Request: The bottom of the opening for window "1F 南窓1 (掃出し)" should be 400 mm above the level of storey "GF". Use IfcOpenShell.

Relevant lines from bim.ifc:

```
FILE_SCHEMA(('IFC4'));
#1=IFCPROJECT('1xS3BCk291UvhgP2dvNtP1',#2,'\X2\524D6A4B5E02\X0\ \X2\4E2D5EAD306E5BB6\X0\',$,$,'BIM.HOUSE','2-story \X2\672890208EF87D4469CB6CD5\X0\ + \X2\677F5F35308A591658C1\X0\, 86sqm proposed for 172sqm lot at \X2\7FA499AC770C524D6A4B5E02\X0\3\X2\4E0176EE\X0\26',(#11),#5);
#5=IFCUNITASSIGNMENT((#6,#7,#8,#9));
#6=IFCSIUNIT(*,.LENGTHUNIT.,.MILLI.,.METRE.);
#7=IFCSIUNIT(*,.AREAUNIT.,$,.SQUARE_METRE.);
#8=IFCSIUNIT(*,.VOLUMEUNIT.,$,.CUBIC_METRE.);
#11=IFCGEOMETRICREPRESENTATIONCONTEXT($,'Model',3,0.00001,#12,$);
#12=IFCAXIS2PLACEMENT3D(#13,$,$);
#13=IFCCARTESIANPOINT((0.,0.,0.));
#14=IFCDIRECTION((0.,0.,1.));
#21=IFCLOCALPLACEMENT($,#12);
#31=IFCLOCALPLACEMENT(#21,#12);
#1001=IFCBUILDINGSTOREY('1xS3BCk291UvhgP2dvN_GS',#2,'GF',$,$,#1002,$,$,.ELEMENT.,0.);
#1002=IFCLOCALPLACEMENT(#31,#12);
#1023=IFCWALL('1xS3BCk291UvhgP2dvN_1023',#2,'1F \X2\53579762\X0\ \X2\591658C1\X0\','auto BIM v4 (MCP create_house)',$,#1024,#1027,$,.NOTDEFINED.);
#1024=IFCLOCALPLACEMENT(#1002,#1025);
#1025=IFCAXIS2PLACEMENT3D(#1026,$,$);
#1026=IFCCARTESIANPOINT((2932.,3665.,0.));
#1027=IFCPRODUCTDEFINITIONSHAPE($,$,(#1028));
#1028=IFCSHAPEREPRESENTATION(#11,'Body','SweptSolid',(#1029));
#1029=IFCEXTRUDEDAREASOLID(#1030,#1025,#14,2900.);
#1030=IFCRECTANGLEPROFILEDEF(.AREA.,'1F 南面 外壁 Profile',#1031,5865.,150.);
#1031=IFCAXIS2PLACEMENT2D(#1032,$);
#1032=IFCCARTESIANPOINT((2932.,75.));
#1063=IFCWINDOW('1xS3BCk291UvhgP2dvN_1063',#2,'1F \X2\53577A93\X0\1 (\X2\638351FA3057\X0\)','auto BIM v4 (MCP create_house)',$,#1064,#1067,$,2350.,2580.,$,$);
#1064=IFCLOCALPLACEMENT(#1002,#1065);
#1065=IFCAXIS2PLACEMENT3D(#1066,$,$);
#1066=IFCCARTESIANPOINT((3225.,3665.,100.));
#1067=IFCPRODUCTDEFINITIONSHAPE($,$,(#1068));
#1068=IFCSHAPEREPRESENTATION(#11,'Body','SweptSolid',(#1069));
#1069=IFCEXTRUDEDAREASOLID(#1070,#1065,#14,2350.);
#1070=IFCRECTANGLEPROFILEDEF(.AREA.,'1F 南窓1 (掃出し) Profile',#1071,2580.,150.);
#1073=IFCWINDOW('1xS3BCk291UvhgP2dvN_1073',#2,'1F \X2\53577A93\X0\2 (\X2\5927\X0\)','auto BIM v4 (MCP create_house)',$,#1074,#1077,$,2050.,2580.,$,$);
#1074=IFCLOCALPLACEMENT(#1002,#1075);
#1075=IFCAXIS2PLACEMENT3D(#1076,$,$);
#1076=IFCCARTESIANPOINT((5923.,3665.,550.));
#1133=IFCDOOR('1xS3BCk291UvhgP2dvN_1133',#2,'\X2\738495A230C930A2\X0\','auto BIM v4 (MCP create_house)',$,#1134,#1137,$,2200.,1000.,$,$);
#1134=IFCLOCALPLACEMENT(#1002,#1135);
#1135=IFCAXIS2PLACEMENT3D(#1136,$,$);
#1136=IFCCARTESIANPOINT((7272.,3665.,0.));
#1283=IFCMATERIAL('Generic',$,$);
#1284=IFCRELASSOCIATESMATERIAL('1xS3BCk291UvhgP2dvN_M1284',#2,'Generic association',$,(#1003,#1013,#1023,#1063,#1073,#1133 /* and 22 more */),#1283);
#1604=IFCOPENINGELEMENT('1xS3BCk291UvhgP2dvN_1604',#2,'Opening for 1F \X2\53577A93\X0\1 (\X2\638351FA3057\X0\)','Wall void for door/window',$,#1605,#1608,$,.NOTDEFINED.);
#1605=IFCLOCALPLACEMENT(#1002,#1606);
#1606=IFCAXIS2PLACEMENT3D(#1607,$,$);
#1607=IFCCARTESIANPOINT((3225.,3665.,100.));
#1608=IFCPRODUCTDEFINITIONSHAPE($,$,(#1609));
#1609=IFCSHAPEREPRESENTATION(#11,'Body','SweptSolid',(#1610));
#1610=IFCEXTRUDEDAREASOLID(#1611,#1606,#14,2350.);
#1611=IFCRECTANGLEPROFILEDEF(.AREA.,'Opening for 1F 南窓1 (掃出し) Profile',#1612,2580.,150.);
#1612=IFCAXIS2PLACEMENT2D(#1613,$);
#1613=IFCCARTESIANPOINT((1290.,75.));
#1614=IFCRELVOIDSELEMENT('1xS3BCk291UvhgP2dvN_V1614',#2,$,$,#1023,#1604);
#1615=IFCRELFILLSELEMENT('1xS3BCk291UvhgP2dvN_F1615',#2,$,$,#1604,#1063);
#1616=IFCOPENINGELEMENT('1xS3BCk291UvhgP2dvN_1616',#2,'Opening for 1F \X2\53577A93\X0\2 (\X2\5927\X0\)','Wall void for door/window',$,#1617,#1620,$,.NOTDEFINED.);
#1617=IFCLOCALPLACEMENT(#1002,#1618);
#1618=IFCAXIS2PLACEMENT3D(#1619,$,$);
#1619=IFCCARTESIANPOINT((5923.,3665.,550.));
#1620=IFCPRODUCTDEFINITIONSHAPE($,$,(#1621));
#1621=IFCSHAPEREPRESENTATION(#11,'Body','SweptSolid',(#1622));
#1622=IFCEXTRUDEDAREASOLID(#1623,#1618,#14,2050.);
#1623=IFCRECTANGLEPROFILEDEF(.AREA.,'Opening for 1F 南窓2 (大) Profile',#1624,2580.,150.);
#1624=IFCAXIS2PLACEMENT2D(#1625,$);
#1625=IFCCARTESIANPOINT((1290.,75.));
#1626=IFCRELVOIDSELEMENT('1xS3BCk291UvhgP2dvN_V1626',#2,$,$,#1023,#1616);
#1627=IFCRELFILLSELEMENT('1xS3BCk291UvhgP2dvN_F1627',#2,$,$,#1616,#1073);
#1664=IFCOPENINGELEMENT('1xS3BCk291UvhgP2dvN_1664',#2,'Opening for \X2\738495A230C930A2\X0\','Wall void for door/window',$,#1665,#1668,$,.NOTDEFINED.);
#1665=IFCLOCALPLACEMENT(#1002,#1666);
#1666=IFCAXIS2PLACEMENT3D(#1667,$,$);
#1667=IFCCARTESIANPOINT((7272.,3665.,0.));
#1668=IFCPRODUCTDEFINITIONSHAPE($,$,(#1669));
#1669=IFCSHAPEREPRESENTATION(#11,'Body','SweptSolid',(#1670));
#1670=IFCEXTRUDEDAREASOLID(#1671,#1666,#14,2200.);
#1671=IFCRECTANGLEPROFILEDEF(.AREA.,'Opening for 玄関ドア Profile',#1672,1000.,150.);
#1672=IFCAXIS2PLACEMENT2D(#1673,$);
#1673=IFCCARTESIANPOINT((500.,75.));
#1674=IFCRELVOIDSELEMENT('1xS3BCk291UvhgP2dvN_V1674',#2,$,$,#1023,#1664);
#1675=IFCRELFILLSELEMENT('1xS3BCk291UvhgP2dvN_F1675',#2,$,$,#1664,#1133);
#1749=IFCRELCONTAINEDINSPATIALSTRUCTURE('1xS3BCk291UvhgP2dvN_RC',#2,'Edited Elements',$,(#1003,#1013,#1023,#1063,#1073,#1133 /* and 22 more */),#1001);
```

```python
import numpy as np
import ifcopenshell
import ifcopenshell.api.geometry
import ifcopenshell.geom
import ifcopenshell.util.element
import ifcopenshell.util.placement
import ifcopenshell.util.shape
import ifcopenshell.util.unit

model = ifcopenshell.open("bim.ifc")
unit_scale = ifcopenshell.util.unit.calculate_unit_scale(model)

window = model.by_guid("1xS3BCk291UvhgP2dvN_1063")
opening = window.FillsVoids[0].RelatingOpeningElement
storey = ifcopenshell.util.element.get_container(window, ifc_class="IfcBuildingStorey")
level = ifcopenshell.util.placement.get_local_placement(storey.ObjectPlacement)[2, 3]

# The opening's origin need not be at the sill, so measure its lowest point.
shape = ifcopenshell.geom.create_shape(ifcopenshell.geom.settings(), opening)
bottom = ifcopenshell.util.shape.get_shape_bottom_elevation(shape, shape.geometry) / unit_scale
dz = level + 400.0 - bottom

shift = np.array([0.0, 0.0, dz])
# The window is not placed relative to its opening, so move both.
for product in (opening, window):
    matrix = ifcopenshell.util.placement.get_local_placement(product.ObjectPlacement)
    matrix[:3, 3] += shift
    ifcopenshell.api.geometry.edit_object_placement(model, product=product, matrix=matrix, is_si=False)

print(f"moved by {dz * unit_scale:+.3f} m")

model.write("bim_edited.ifc")
```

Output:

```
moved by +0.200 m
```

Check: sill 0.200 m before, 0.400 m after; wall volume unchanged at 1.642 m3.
